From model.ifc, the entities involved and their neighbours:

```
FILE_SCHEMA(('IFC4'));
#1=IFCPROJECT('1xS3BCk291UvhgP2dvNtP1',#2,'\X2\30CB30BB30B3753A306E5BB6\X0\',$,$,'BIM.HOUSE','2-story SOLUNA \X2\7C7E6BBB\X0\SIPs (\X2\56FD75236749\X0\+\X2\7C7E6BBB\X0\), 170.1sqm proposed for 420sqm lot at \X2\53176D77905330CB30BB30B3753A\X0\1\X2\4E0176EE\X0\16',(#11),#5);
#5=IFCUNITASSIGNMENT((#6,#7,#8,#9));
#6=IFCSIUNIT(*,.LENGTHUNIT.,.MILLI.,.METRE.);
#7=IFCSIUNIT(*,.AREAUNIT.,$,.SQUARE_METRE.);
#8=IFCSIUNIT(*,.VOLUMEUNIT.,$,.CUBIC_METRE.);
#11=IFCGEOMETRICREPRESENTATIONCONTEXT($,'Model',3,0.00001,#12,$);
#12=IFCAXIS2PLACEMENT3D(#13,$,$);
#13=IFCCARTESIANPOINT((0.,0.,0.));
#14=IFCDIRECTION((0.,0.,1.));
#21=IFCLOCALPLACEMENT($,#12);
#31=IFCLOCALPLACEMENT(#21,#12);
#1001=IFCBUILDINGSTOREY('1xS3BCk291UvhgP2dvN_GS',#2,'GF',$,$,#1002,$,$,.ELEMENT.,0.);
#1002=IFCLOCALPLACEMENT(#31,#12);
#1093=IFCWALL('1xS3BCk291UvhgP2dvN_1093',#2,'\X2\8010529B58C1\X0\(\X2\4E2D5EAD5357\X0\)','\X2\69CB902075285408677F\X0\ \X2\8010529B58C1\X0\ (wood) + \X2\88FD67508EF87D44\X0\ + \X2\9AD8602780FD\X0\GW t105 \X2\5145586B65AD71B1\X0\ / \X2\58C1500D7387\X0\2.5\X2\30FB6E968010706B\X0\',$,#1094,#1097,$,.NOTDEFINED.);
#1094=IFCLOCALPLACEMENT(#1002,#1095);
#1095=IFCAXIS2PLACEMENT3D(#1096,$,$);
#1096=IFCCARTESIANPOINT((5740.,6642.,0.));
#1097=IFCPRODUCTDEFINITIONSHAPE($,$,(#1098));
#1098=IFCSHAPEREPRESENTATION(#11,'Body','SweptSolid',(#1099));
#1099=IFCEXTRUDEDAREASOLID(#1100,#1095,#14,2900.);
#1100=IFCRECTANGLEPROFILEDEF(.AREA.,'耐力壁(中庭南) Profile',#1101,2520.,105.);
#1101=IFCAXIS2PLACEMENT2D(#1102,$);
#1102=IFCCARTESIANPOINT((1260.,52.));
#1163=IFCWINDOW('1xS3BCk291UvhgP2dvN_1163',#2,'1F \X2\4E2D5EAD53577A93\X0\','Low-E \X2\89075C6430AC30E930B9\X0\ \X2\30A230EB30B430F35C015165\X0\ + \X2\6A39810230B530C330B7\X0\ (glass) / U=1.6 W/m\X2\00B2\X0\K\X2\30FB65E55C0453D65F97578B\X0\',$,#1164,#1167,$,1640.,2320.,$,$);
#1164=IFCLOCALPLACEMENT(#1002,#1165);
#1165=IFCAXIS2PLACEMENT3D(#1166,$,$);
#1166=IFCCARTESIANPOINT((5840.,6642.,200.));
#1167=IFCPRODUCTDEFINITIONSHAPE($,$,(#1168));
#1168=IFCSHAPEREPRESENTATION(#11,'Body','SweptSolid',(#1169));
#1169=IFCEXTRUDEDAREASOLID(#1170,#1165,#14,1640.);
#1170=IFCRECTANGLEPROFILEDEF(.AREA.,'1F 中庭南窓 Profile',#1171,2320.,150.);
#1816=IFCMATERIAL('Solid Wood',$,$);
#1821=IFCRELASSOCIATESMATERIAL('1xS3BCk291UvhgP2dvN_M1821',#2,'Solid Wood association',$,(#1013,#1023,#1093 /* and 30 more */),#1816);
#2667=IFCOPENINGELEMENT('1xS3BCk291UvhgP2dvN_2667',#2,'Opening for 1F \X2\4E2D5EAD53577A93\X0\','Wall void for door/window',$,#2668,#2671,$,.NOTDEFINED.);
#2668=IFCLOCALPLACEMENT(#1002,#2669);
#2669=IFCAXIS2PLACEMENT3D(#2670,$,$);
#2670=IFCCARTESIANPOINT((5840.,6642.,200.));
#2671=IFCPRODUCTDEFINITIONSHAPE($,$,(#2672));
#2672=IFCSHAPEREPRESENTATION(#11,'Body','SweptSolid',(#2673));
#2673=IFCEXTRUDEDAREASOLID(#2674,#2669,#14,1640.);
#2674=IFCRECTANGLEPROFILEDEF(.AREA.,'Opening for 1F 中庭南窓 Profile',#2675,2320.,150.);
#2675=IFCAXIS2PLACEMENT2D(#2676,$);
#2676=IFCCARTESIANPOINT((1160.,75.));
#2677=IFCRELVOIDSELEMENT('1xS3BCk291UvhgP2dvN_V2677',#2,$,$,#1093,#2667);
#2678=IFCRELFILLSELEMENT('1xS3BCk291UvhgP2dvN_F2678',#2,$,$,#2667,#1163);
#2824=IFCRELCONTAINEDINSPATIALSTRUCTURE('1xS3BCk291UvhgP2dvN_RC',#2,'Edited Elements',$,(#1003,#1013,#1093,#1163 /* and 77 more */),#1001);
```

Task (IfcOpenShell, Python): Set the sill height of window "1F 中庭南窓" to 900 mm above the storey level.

```python
import numpy as np
import ifcopenshell
import ifcopenshell.api.geometry
import ifcopenshell.geom
import ifcopenshell.util.element
import ifcopenshell.util.placement
import ifcopenshell.util.shape
import ifcopenshell.util.unit

model = ifcopenshell.open("model.ifc")
unit_scale = ifcopenshell.util.unit.calculate_unit_scale(model)

window = model.by_guid("1xS3BCk291UvhgP2dvN_1163")
opening = window.FillsVoids[0].RelatingOpeningElement
storey = ifcopenshell.util.element.get_container(window, ifc_class="IfcBuildingStorey")
level = ifcopenshell.util.placement.get_local_placement(storey.ObjectPlacement)[2, 3]

# The opening's origin need not be at the sill, so measure its lowest point.
shape = ifcopenshell.geom.create_shape(ifcopenshell.geom.settings(), opening)
bottom = ifcopenshell.util.shape.get_shape_bottom_elevation(shape, shape.geometry) / unit_scale
dz = level + 0.9 / unit_scale - bottom

shift = np.array([0.0, 0.0, dz])
# The window is not placed relative to its opening, so move both.
for product in (opening, window):
    matrix = ifcopenshell.util.placement.get_local_placement(product.ObjectPlacement)
    matrix[:3, 3] += shift
    ifcopenshell.api.geometry.edit_object_placement(model, product=product, matrix=matrix, is_si=False)

print(f"moved by {dz * unit_scale:+.3f} m")

model.write("model_edited.ifc")
```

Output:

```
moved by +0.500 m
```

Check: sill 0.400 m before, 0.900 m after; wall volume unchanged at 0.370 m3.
